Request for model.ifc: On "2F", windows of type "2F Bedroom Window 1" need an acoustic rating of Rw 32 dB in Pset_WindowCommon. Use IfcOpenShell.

First a look at what the model holds.

```python
import ifcopenshell
import ifcopenshell.util.element

model = ifcopenshell.open("model.ifc")
print(model.schema)
storey = next(s for s in model.by_type("IfcBuildingStorey") if s.Name == "2F")
windows = [e for e in ifcopenshell.util.element.get_decomposition(storey) if e.is_a("IfcWindow")]
seen = {}
for e in windows:
    element_type = ifcopenshell.util.element.get_type(e)
    key = (element_type.Name if element_type != e and element_type else None, ifcopenshell.util.element.get_pset(e, "Pset_WindowCommon", "AcousticRating"))
    seen[key] = seen.get(key, 0) + 1
for (name, value), count in sorted(seen.items(), key=str):
    print(count, "x", name, "|", value)
```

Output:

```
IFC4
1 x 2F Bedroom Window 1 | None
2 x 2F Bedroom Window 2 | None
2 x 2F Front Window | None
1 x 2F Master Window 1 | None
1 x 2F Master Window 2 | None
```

```python
import ifcopenshell
import ifcopenshell.api.pset
import ifcopenshell.util.element

model = ifcopenshell.open("model.ifc")

storey = next(s for s in model.by_type("IfcBuildingStorey") if s.Name == "2F")
windows = [e for e in ifcopenshell.util.element.get_decomposition(storey) if e.is_a("IfcWindow")]

count = 0
for e in windows:
    element_type = ifcopenshell.util.element.get_type(e)
    if element_type in (None, e) or element_type.Name != "2F Bedroom Window 1":
        continue
    # add_pset returns the element's existing set when there is one.
    pset = ifcopenshell.api.pset.add_pset(model, product=e, name="Pset_WindowCommon")
    ifcopenshell.api.pset.edit_pset(model, pset=pset, properties={"AcousticRating": "Rw 32 dB"})
    count += 1

print(count, "windows updated")

model.write("model-out.ifc")
```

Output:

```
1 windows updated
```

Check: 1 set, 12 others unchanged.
